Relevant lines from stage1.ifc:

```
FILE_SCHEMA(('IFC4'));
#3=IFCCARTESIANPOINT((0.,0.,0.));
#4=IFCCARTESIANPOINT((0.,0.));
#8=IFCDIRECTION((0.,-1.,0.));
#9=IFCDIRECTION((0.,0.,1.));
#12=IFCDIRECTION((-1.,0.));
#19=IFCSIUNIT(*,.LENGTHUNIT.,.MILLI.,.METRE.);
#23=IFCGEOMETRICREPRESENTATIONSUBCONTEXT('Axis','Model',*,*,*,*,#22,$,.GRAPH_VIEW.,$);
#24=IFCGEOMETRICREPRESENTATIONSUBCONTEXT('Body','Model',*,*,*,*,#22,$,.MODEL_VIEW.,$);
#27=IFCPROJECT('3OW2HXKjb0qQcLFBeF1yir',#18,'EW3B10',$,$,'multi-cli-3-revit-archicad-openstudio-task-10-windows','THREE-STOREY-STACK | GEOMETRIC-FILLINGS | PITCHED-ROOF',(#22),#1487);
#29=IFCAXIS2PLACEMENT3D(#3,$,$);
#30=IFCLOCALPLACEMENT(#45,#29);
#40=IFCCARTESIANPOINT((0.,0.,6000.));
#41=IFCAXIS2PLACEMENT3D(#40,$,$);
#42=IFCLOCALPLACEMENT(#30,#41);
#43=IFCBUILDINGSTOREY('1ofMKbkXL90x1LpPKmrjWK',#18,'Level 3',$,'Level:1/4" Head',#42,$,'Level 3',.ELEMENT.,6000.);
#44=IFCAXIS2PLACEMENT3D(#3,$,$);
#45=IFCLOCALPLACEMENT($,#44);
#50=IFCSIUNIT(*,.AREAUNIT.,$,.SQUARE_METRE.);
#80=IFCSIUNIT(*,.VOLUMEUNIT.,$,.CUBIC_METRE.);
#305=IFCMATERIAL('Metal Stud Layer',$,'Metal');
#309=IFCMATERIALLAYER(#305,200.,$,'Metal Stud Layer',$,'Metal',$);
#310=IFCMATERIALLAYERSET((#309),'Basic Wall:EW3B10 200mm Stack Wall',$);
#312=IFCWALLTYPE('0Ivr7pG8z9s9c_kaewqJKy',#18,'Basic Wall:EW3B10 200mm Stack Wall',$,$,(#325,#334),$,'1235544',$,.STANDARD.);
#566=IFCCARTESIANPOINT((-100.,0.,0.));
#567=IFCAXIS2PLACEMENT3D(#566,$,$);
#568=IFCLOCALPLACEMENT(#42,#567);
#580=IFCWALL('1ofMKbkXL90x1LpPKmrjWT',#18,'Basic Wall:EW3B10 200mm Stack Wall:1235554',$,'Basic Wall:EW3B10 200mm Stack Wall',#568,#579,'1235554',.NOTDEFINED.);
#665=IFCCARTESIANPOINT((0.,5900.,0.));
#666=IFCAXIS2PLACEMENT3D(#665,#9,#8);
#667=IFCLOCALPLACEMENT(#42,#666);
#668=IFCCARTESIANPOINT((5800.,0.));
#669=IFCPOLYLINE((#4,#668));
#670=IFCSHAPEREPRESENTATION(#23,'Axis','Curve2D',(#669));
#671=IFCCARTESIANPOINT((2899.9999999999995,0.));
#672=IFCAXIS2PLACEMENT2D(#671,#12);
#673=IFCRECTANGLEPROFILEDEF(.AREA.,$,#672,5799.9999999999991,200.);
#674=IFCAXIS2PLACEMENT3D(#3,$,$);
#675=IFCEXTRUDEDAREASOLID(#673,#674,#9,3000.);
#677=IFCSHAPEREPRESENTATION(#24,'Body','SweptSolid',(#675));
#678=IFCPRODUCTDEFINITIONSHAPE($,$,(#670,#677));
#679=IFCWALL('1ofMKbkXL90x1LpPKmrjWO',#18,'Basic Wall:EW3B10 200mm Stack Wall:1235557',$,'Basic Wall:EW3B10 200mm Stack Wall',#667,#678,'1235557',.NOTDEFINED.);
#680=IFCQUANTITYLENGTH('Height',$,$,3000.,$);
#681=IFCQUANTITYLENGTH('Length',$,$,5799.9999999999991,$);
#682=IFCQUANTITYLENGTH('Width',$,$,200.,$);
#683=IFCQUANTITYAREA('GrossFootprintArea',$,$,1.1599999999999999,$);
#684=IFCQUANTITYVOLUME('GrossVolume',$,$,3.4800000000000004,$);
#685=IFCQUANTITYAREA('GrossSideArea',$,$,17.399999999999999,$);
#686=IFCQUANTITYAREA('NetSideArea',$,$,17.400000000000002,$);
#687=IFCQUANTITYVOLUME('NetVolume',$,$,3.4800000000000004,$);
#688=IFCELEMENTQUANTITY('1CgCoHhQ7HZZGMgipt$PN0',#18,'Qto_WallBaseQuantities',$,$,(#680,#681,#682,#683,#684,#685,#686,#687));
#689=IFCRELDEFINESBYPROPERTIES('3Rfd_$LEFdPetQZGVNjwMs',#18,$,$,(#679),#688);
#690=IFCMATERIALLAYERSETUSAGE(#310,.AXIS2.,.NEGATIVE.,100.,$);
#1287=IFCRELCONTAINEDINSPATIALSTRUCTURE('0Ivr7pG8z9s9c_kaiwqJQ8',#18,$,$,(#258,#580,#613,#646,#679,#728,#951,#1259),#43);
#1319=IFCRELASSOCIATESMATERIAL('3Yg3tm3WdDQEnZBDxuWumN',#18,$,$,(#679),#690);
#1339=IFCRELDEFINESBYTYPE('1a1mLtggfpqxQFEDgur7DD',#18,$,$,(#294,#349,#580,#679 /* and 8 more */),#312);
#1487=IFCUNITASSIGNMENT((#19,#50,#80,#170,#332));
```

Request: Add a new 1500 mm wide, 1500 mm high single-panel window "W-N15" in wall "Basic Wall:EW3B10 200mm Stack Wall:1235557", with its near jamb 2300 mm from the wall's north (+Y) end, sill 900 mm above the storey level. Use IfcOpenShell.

```python
import numpy as np
import ifcopenshell
import ifcopenshell.api.feature
import ifcopenshell.api.geometry
import ifcopenshell.api.pset
import ifcopenshell.api.root
import ifcopenshell.api.spatial
import ifcopenshell.geom
import ifcopenshell.util.element
import ifcopenshell.util.placement
import ifcopenshell.util.representation
import ifcopenshell.util.shape
import ifcopenshell.util.unit

model = ifcopenshell.open("stage1.ifc")
unit_scale = ifcopenshell.util.unit.calculate_unit_scale(model)
area_scale = ifcopenshell.util.unit.calculate_unit_scale(model, "AREAUNIT")
volume_scale = ifcopenshell.util.unit.calculate_unit_scale(model, "VOLUMEUNIT")
settings = ifcopenshell.geom.settings()


def volume(element):
    """Net volume in cubic metres, openings subtracted."""
    shape = ifcopenshell.geom.create_shape(settings, element)
    return ifcopenshell.util.shape.get_volume(shape.geometry)


wall = model.by_guid("1ofMKbkXL90x1LpPKmrjWO")
storey = ifcopenshell.util.element.get_container(wall, ifc_class="IfcBuildingStorey")
context = ifcopenshell.util.representation.get_context(model, "Model", "Body", "MODEL_VIEW")
before = volume(wall)

width, height, from_end, sill = 1.5, 1.5, 2.3, 0.9  # metres

# The wall runs along its own X axis, and the end named is its -X end.
wall_shape = ifcopenshell.geom.create_shape(settings, wall)
x, y, z = ifcopenshell.util.shape.get_vertices(wall_shape.geometry).T
start = x.min() + from_end
face, thickness = float(y.min()), float(y.max() - y.min())
wall_matrix = ifcopenshell.util.placement.get_local_placement(wall.ObjectPlacement)
level = ifcopenshell.util.placement.get_local_placement(storey.ObjectPlacement)[2, 3]


def in_wall(x, y):
    """Placement at x, y metres in the wall's axes, at sill height."""
    matrix = wall_matrix.copy()
    matrix[:, 3] = wall_matrix @ np.array([x / unit_scale, y / unit_scale, 0.0, 1.0])
    matrix[2, 3] = level + sill / unit_scale
    return matrix


# Opening: a box that overshoots both wall faces by 50 mm.
opening = ifcopenshell.api.root.create_entity(model, ifc_class="IfcOpeningElement", predefined_type="OPENING")
box = ifcopenshell.api.geometry.add_wall_representation(
    model, context=context, length=width, height=height, thickness=thickness + 0.1
)
ifcopenshell.api.geometry.assign_representation(model, product=opening, representation=box)
ifcopenshell.api.geometry.edit_object_placement(model, product=opening, matrix=in_wall(start, face - 0.05), is_si=False)
ifcopenshell.api.feature.add_feature(model, feature=opening, element=wall)

window = ifcopenshell.api.root.create_entity(model, ifc_class="IfcWindow", name="W-N15", predefined_type="WINDOW")
window.OverallWidth, window.OverallHeight = width / unit_scale, height / unit_scale
window.PartitioningType = "SINGLE_PANEL"
body = ifcopenshell.api.geometry.add_window_representation(
    model,
    context=context,
    overall_width=window.OverallWidth,
    overall_height=window.OverallHeight,
    partition_type="SINGLE_PANEL",
)
ifcopenshell.api.geometry.assign_representation(model, product=window, representation=body)
ifcopenshell.api.spatial.assign_container(model, products=[window], relating_structure=storey)
ifcopenshell.api.feature.add_filling(model, opening=opening, element=window)

# Centre the window in the wall's thickness.
ifcopenshell.api.geometry.edit_object_placement(model, product=window, matrix=in_wall(start, face), is_si=False)
window_shape = ifcopenshell.geom.create_shape(settings, window)
depth = ifcopenshell.util.shape.get_vertices(window_shape.geometry)[:, 1]
offset = face + thickness / 2 - (depth.min() + depth.max()) / 2
ifcopenshell.api.geometry.edit_object_placement(model, product=window, matrix=in_wall(start, offset), is_si=False)

after = volume(wall)

# Update the wall's stored quantities.
qto = model.by_id(ifcopenshell.util.element.get_pset(wall, "Qto_WallBaseQuantities", should_inherit=False)["id"])
ifcopenshell.api.pset.edit_qto(model, qto=qto, properties={
    "NetSideArea": after / thickness / area_scale,
    "NetVolume": after / volume_scale,
})

print(f"wall volume {before:.3f} -> {after:.3f} m3")

model.write("stage1-out.ifc")
```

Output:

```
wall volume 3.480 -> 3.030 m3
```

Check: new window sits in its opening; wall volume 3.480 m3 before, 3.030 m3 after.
